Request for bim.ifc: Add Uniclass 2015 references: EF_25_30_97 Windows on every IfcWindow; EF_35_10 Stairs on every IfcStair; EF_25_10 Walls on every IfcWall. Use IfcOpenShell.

First a look at what the model holds.

```python
import ifcopenshell

model = ifcopenshell.open("bim.ifc")
print(model.schema)
print("classifications:", [c.Name for c in model.by_type("IfcClassification")])
for ifc_class in ("IfcDoor", "IfcRoof", "IfcStair", "IfcWall", "IfcWindow"):
    print(ifc_class, len(model.by_type(ifc_class)))
```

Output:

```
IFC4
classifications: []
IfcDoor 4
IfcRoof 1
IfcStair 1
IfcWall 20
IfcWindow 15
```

```python
import ifcopenshell
import ifcopenshell.api.classification

model = ifcopenshell.open("bim.ifc")

system = ifcopenshell.api.classification.add_classification(model, classification="Uniclass 2015")

codes = {
    "IfcWindow": ("EF_25_30_97", "Windows"),
    "IfcStair": ("EF_35_10", "Stairs"),
    "IfcWall": ("EF_25_10", "Walls"),
}
for ifc_class, (code, name) in codes.items():
    products = model.by_type(ifc_class)
    ifcopenshell.api.classification.add_reference(
        model, products=products, classification=system, identification=code, name=name
    )
    print(code, len(products))

model.write("bim_rev.ifc")
```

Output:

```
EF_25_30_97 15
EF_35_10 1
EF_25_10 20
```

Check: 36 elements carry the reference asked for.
